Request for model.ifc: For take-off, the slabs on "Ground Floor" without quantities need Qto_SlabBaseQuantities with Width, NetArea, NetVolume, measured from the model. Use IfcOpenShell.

First a look at what the model holds.

```python
import ifcopenshell
import ifcopenshell.util.element
import ifcopenshell.util.unit

model = ifcopenshell.open("model.ifc")
print(model.schema)
for unit_type in ("LENGTHUNIT", "AREAUNIT", "VOLUMEUNIT"):
    print(unit_type, ifcopenshell.util.unit.calculate_unit_scale(model, unit_type))
storey = next(s for s in model.by_type("IfcBuildingStorey") if s.Name == "Ground Floor")
slabs = [e for e in ifcopenshell.util.element.get_decomposition(storey) if e.is_a("IfcSlab")]
for e in sorted(slabs, key=lambda e: e.id()):
    print(e.id(), e.is_a(), e.Name, list(ifcopenshell.util.element.get_psets(e, qtos_only=True)), sep=" | ")
```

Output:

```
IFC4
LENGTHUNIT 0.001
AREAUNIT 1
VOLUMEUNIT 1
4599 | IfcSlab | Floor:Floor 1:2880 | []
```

```python
import ifcopenshell
import ifcopenshell.api.pset
import ifcopenshell.geom
import ifcopenshell.util.element
import ifcopenshell.util.shape
import ifcopenshell.util.unit

model = ifcopenshell.open("model.ifc")
unit_scale = ifcopenshell.util.unit.calculate_unit_scale(model)
area_scale = ifcopenshell.util.unit.calculate_unit_scale(model, "AREAUNIT")
volume_scale = ifcopenshell.util.unit.calculate_unit_scale(model, "VOLUMEUNIT")
settings = ifcopenshell.geom.settings()

storey = next(s for s in model.by_type("IfcBuildingStorey") if s.Name == "Ground Floor")
slabs = [e for e in ifcopenshell.util.element.get_decomposition(storey) if e.is_a("IfcSlab")]

for e in sorted(slabs, key=lambda e: e.id()):
    if ifcopenshell.util.element.get_psets(e, qtos_only=True, should_inherit=False):
        continue
    # Geometry comes back in metres, in the element's own axes.
    shape = ifcopenshell.geom.create_shape(settings, e)
    values = {
        "Width": ifcopenshell.util.shape.get_z(shape.geometry) / unit_scale,
        "NetArea": ifcopenshell.util.shape.get_footprint_area(shape.geometry) / area_scale,
        "NetVolume": ifcopenshell.util.shape.get_volume(shape.geometry) / volume_scale,
    }
    qto = ifcopenshell.api.pset.add_qto(model, product=e, name="Qto_SlabBaseQuantities")
    ifcopenshell.api.pset.edit_qto(model, qto=qto, properties=values)
    print(e.id(), {k: round(v, 3) for k, v in values.items()})

model.write("model-out.ifc")
```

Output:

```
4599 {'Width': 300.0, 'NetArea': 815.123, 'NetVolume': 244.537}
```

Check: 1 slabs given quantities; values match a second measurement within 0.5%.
